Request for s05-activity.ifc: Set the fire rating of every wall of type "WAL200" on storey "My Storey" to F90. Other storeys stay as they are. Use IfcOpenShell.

First a look at what the model holds.

```python
import ifcopenshell
import ifcopenshell.util.element

model = ifcopenshell.open("s05-activity.ifc")
print(model.schema)
storey = next(s for s in model.by_type("IfcBuildingStorey") if s.Name == "My Storey")
walls = [e for e in ifcopenshell.util.element.get_decomposition(storey) if e.is_a("IfcWall")]
seen = {}
for e in walls:
    element_type = ifcopenshell.util.element.get_type(e)
    key = (element_type.Name if element_type != e and element_type else None, ifcopenshell.util.element.get_pset(e, "Pset_WallCommon", "FireRating"))
    seen[key] = seen.get(key, 0) + 1
for (name, value), count in sorted(seen.items(), key=str):
    print(count, "x", name, "|", value)
```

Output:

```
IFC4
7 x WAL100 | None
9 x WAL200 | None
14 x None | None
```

```python
import ifcopenshell
import ifcopenshell.api.pset
import ifcopenshell.util.element

model = ifcopenshell.open("s05-activity.ifc")

storey = next(s for s in model.by_type("IfcBuildingStorey") if s.Name == "My Storey")
walls = [e for e in ifcopenshell.util.element.get_decomposition(storey) if e.is_a("IfcWall")]

count = 0
for e in walls:
    element_type = ifcopenshell.util.element.get_type(e)
    if element_type in (None, e) or element_type.Name != "WAL200":
        continue
    # add_pset returns the element's existing set when there is one.
    pset = ifcopenshell.api.pset.add_pset(model, product=e, name="Pset_WallCommon")
    ifcopenshell.api.pset.edit_pset(model, pset=pset, properties={"FireRating": "F90"})
    count += 1

print(count, "walls updated")

model.write("s05-activity-out.ifc")
```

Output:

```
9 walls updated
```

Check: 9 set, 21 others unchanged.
